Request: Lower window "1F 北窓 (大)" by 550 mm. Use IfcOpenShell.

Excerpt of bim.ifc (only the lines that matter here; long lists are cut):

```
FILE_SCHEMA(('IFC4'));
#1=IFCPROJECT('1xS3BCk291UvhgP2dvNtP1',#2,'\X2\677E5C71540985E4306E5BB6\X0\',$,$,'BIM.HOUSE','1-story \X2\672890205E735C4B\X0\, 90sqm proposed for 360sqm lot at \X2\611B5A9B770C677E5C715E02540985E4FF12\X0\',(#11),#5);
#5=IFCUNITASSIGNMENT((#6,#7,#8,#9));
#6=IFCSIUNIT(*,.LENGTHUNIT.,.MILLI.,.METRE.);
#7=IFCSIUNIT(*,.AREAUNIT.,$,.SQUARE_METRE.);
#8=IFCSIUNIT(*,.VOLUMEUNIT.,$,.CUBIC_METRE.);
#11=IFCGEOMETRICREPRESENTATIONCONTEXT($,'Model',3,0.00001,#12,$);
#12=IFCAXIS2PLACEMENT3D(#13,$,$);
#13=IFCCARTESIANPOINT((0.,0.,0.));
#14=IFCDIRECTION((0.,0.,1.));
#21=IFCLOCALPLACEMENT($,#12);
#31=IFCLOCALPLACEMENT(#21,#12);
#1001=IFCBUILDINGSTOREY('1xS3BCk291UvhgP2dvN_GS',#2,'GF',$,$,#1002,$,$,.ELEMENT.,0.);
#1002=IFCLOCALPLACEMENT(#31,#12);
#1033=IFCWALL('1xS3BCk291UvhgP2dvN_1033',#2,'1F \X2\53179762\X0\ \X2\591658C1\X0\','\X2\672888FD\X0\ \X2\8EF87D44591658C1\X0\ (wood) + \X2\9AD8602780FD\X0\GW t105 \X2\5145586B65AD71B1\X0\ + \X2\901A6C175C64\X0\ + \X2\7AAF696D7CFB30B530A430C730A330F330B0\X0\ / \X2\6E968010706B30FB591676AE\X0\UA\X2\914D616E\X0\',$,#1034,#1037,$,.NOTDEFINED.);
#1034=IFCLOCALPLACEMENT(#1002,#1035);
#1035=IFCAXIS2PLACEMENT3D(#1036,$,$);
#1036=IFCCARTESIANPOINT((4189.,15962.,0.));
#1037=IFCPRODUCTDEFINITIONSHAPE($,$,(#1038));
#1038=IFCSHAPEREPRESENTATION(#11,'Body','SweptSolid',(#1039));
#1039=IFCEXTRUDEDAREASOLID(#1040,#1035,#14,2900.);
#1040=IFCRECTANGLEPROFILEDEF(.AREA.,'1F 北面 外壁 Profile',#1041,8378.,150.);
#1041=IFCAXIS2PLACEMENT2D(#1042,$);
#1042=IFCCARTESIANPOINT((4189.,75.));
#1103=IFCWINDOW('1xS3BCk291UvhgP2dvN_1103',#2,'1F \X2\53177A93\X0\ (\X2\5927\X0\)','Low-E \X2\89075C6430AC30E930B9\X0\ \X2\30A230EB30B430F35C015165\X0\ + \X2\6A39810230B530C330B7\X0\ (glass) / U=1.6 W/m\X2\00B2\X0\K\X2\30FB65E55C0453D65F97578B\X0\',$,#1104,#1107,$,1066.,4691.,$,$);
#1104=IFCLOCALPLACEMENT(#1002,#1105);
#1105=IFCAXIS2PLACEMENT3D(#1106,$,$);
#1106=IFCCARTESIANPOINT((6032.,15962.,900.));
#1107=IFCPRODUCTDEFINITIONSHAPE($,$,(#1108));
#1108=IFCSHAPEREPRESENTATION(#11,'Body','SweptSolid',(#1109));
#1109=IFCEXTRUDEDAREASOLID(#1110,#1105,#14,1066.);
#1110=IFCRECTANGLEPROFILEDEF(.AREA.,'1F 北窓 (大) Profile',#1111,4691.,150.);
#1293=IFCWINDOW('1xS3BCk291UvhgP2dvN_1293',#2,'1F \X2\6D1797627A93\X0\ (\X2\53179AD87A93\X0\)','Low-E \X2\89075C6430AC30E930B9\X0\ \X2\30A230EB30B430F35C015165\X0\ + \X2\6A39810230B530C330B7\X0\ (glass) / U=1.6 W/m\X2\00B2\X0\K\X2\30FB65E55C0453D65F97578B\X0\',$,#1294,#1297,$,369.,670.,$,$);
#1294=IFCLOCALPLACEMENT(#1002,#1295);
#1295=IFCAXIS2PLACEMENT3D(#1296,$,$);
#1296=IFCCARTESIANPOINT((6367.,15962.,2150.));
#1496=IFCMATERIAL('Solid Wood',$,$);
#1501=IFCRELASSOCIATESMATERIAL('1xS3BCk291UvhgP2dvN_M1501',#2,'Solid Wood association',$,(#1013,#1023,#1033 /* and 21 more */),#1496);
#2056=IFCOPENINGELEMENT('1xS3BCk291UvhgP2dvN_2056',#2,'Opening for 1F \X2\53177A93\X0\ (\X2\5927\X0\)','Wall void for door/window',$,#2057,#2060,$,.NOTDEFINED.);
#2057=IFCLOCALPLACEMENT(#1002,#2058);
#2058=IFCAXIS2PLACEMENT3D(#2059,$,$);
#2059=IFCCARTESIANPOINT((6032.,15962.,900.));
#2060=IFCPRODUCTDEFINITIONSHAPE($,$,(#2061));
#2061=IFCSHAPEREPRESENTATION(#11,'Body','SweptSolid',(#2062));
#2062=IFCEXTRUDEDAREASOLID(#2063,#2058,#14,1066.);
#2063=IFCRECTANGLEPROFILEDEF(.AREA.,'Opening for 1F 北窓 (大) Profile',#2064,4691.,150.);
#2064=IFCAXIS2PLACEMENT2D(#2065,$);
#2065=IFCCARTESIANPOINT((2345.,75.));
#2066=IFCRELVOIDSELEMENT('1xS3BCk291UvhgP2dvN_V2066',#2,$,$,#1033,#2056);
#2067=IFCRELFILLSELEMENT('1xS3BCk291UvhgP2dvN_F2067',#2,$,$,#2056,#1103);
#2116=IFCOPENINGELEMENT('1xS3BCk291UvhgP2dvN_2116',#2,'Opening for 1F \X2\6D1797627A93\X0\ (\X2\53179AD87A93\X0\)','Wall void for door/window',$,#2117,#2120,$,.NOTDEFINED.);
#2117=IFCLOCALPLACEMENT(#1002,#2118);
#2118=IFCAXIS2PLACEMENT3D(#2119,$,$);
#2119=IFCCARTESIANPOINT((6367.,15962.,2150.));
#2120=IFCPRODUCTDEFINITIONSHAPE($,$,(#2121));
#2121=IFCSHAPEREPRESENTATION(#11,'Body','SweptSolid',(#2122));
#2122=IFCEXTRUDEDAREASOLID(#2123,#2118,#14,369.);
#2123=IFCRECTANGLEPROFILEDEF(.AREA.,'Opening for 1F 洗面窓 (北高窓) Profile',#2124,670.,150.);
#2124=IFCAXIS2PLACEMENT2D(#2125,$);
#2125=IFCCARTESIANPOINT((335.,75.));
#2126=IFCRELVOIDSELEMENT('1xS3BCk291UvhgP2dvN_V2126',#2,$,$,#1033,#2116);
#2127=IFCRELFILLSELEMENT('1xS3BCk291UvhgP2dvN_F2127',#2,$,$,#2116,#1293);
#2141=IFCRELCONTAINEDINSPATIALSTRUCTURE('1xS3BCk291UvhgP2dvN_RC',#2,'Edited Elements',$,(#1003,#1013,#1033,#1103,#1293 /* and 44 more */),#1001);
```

```python
import numpy as np
import ifcopenshell
import ifcopenshell.api.geometry
import ifcopenshell.util.placement
import ifcopenshell.util.unit

model = ifcopenshell.open("bim.ifc")
unit_scale = ifcopenshell.util.unit.calculate_unit_scale(model)

window = model.by_guid("1xS3BCk291UvhgP2dvN_1103")
opening = window.FillsVoids[0].RelatingOpeningElement
dz = -550.0

shift = np.array([0.0, 0.0, dz])
# The window is not placed relative to its opening, so move both.
for product in (opening, window):
    matrix = ifcopenshell.util.placement.get_local_placement(product.ObjectPlacement)
    matrix[:3, 3] += shift
    ifcopenshell.api.geometry.edit_object_placement(model, product=product, matrix=matrix, is_si=False)

print(f"moved by {dz * unit_scale:+.3f} m")

model.write("bim_updated.ifc")
```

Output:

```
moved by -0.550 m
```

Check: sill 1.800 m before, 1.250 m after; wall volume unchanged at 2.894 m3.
